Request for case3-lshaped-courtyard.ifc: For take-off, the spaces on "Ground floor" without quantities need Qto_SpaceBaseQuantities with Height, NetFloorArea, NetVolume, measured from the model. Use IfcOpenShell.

First a look at what the model holds.

```python
import ifcopenshell
import ifcopenshell.util.element
import ifcopenshell.util.unit

model = ifcopenshell.open("case3-lshaped-courtyard.ifc")
print(model.schema)
for unit_type in ("LENGTHUNIT", "AREAUNIT", "VOLUMEUNIT"):
    print(unit_type, ifcopenshell.util.unit.calculate_unit_scale(model, unit_type))
storey = next(s for s in model.by_type("IfcBuildingStorey") if s.Name == "Ground floor")
spaces = [e for e in ifcopenshell.util.element.get_decomposition(storey) if e.is_a("IfcSpace")]
for e in sorted(spaces, key=lambda e: e.id()):
    print(e.id(), e.is_a(), e.Name, list(ifcopenshell.util.element.get_psets(e, qtos_only=True)), sep=" | ")
```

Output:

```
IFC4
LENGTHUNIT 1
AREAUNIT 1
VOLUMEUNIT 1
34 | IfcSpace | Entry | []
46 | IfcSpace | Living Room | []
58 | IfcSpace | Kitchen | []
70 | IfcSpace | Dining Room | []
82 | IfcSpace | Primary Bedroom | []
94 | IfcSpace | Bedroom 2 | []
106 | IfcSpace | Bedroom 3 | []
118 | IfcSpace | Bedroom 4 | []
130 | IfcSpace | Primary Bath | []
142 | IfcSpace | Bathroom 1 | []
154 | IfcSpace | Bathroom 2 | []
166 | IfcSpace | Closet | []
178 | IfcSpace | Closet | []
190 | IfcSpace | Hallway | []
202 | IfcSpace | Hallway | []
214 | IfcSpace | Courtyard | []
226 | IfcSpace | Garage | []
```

```python
import ifcopenshell
import ifcopenshell.api.pset
import ifcopenshell.geom
import ifcopenshell.util.element
import ifcopenshell.util.shape
import ifcopenshell.util.unit

model = ifcopenshell.open("case3-lshaped-courtyard.ifc")
unit_scale = ifcopenshell.util.unit.calculate_unit_scale(model)
area_scale = ifcopenshell.util.unit.calculate_unit_scale(model, "AREAUNIT")
volume_scale = ifcopenshell.util.unit.calculate_unit_scale(model, "VOLUMEUNIT")
settings = ifcopenshell.geom.settings()

storey = next(s for s in model.by_type("IfcBuildingStorey") if s.Name == "Ground floor")
spaces = [e for e in ifcopenshell.util.element.get_decomposition(storey) if e.is_a("IfcSpace")]

for e in sorted(spaces, key=lambda e: e.id()):
    if ifcopenshell.util.element.get_psets(e, qtos_only=True, should_inherit=False):
        continue
    # Geometry comes back in metres, in the element's own axes.
    shape = ifcopenshell.geom.create_shape(settings, e)
    values = {
        "Height": ifcopenshell.util.shape.get_z(shape.geometry) / unit_scale,
        "NetFloorArea": ifcopenshell.util.shape.get_footprint_area(shape.geometry) / area_scale,
        "NetVolume": ifcopenshell.util.shape.get_volume(shape.geometry) / volume_scale,
    }
    qto = ifcopenshell.api.pset.add_qto(model, product=e, name="Qto_SpaceBaseQuantities")
    ifcopenshell.api.pset.edit_qto(model, qto=qto, properties=values)
    print(e.id(), {k: round(v, 3) for k, v in values.items()})

model.write("case3-lshaped-courtyard_updated.ifc")
```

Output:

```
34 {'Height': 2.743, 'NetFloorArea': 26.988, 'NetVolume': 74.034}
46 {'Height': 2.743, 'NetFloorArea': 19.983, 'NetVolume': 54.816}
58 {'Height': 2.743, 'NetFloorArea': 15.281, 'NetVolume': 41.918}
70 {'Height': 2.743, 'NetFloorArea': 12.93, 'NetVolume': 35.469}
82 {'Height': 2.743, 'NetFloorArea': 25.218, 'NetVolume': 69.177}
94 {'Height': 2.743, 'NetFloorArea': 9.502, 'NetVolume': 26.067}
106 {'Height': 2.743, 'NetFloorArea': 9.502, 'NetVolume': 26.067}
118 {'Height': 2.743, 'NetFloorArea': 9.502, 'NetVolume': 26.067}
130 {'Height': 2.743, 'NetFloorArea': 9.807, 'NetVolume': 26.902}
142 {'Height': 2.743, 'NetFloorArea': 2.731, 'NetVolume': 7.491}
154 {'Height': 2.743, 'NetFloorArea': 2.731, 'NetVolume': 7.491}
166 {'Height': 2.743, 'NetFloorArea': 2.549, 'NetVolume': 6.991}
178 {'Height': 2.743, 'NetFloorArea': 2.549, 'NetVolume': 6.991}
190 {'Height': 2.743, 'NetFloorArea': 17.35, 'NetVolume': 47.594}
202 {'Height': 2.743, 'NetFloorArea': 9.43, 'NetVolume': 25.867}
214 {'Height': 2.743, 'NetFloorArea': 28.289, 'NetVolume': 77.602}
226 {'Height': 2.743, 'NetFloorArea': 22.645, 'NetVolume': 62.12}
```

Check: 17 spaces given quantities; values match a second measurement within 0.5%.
